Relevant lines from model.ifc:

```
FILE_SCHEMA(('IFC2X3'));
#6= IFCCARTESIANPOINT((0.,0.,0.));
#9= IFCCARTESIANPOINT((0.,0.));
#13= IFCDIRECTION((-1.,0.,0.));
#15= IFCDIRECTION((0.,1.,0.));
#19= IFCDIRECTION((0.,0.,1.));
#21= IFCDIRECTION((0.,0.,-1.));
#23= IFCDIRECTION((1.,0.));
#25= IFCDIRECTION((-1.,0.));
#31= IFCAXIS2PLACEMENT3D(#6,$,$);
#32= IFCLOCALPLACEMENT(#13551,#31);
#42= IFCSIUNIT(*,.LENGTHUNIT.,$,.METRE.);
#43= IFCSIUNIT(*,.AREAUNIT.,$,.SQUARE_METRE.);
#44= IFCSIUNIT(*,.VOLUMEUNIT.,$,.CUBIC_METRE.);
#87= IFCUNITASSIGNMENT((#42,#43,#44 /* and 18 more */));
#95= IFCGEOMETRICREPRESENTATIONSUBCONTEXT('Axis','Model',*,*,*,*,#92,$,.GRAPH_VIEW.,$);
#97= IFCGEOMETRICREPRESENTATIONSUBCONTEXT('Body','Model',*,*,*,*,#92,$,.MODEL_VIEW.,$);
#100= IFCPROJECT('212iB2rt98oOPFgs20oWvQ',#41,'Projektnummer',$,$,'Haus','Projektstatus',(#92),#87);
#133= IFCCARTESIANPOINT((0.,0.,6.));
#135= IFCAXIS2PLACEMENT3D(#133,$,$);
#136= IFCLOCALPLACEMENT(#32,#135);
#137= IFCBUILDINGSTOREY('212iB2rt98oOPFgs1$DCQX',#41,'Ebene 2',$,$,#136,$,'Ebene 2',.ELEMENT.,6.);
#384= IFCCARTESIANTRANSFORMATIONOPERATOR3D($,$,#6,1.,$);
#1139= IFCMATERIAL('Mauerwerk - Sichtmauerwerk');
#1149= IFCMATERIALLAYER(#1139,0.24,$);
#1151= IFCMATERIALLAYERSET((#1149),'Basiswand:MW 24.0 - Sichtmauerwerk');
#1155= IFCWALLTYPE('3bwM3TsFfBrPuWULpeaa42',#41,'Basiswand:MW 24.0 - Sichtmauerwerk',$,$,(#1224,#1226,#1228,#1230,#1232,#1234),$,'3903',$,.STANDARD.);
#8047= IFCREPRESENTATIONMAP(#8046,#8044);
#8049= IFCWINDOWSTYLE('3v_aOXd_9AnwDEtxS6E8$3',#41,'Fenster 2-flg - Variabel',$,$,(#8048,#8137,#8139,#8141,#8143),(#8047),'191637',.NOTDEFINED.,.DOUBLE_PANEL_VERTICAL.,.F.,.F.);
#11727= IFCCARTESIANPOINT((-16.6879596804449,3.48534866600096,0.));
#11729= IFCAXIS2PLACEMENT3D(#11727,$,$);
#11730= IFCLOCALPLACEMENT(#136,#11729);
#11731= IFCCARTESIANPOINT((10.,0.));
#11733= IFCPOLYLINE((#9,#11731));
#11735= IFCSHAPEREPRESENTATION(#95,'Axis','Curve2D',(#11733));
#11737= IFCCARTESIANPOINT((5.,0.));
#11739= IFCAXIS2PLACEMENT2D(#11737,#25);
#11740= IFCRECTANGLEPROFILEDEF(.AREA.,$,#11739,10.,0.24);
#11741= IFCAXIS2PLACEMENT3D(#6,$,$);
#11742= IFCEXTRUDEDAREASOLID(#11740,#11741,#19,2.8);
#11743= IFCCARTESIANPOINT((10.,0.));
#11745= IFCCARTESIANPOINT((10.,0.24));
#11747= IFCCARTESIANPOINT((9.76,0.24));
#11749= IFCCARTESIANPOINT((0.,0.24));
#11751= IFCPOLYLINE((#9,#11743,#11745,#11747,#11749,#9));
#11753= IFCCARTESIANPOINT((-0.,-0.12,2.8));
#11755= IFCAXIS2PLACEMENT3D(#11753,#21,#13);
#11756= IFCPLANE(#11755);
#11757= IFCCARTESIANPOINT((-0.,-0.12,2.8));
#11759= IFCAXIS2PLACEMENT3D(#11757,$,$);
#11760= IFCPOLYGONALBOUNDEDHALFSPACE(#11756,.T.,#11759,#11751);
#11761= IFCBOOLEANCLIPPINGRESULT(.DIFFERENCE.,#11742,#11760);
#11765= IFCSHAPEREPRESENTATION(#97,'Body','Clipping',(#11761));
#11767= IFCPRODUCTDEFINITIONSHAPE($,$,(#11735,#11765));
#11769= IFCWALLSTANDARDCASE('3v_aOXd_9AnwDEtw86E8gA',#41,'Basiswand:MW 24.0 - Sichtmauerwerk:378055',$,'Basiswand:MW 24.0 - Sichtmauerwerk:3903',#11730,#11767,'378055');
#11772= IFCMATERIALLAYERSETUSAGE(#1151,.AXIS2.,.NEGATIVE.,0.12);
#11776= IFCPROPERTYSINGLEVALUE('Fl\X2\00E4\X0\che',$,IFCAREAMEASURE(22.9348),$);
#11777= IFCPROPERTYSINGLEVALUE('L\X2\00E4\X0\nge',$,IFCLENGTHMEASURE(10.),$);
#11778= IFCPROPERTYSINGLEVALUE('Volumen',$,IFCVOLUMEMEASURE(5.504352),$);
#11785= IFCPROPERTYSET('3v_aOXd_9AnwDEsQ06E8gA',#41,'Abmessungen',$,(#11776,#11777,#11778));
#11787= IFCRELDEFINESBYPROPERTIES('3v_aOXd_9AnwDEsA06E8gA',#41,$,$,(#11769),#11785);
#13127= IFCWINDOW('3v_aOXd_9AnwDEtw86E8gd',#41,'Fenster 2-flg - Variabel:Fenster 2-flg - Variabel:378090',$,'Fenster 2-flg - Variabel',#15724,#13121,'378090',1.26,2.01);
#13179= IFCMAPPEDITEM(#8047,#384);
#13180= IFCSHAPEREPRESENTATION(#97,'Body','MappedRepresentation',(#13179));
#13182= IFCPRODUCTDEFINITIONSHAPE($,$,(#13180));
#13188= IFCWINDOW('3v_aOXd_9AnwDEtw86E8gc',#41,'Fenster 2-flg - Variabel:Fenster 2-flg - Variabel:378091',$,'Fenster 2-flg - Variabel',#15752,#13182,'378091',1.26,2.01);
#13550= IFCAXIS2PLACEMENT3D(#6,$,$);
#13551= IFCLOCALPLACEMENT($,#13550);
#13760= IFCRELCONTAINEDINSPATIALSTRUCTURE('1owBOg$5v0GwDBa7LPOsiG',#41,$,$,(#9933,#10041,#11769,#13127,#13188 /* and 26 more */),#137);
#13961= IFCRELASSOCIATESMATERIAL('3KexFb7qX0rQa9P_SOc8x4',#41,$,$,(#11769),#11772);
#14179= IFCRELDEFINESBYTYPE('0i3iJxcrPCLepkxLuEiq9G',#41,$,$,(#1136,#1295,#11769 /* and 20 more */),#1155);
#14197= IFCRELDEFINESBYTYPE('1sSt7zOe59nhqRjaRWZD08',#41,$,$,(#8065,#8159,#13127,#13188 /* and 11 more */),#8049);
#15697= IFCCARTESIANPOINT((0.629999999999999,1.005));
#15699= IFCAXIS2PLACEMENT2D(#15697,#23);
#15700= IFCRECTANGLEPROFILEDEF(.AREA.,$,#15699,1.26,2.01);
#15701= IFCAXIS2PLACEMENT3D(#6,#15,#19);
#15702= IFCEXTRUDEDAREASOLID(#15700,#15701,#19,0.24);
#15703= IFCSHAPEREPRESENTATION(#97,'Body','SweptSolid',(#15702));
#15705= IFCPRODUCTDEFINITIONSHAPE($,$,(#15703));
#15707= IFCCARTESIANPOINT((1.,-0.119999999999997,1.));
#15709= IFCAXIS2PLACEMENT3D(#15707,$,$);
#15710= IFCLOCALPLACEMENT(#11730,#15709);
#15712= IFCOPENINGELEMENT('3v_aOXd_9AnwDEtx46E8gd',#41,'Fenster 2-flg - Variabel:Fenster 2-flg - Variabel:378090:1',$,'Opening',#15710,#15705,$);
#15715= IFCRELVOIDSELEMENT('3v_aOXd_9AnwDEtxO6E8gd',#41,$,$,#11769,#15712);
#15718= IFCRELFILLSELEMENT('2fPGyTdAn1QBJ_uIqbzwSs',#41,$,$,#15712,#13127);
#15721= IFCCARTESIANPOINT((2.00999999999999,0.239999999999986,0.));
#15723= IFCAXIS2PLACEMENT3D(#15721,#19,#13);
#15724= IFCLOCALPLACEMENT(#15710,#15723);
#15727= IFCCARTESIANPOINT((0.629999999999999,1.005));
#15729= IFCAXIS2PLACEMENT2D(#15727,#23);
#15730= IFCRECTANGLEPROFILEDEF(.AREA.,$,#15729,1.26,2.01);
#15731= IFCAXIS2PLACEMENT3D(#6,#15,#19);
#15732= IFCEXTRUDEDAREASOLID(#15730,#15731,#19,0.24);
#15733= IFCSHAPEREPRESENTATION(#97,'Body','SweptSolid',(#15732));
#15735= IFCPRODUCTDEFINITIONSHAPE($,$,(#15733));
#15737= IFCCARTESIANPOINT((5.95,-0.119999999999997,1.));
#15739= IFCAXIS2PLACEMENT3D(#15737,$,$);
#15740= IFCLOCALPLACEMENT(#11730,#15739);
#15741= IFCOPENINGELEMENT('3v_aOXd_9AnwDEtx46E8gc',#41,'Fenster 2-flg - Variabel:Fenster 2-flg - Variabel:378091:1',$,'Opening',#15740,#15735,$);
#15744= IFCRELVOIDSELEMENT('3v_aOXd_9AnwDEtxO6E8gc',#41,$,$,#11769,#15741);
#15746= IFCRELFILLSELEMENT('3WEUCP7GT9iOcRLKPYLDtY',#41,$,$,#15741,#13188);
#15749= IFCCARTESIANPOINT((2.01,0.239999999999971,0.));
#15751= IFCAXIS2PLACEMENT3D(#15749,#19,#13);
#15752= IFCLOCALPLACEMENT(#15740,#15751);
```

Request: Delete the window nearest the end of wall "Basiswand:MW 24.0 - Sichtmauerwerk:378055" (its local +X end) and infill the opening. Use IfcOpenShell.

```python
import ifcopenshell
import ifcopenshell.api.feature
import ifcopenshell.api.pset
import ifcopenshell.api.root
import ifcopenshell.geom
import ifcopenshell.util.element
import ifcopenshell.util.shape
import ifcopenshell.util.unit

model = ifcopenshell.open("model.ifc")
area_scale = ifcopenshell.util.unit.calculate_unit_scale(model, "AREAUNIT")
volume_scale = ifcopenshell.util.unit.calculate_unit_scale(model, "VOLUMEUNIT")
settings = ifcopenshell.geom.settings()


def volume(element):
    """Net volume in cubic metres, openings subtracted."""
    shape = ifcopenshell.geom.create_shape(settings, element)
    return ifcopenshell.util.shape.get_volume(shape.geometry)


window = model.by_guid("3v_aOXd_9AnwDEtw86E8gc")
opening = window.FillsVoids[0].RelatingOpeningElement
wall = opening.VoidsElements[0].RelatingBuildingElement
before = volume(wall)

ifcopenshell.api.root.remove_product(model, product=window)
ifcopenshell.api.feature.remove_feature(model, feature=opening)

after = volume(wall)
thickness = 0.24  # wall thickness in metres

# Update the wall's stored quantities.
pset = model.by_id(ifcopenshell.util.element.get_pset(wall, "Abmessungen", should_inherit=False)["id"])
ifcopenshell.api.pset.edit_pset(model, pset=pset, properties={
    "Fläche": model.create_entity("IfcAreaMeasure", after / thickness / area_scale),
    "Volumen": model.create_entity("IfcVolumeMeasure", after / volume_scale),
})

print(f"wall volume {before:.3f} -> {after:.3f} m3")

model.write("model_rev.ifc")
```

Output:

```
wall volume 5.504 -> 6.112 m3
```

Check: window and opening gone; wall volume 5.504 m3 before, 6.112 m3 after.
